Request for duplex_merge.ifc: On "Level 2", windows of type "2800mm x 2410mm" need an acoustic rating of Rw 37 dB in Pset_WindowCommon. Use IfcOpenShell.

First a look at what the model holds.

```python
import ifcopenshell
import ifcopenshell.util.element

model = ifcopenshell.open("duplex_merge.ifc")
print(model.schema)
storey = next(s for s in model.by_type("IfcBuildingStorey") if s.Name == "Level 2")
windows = [e for e in ifcopenshell.util.element.get_decomposition(storey) if e.is_a("IfcWindow")]
seen = {}
for e in windows:
    element_type = ifcopenshell.util.element.get_type(e)
    key = (element_type.Name if element_type != e and element_type else None, ifcopenshell.util.element.get_pset(e, "Pset_WindowCommon", "AcousticRating"))
    seen[key] = seen.get(key, 0) + 1
for (name, value), count in sorted(seen.items(), key=str):
    print(count, "x", name, "|", value)
```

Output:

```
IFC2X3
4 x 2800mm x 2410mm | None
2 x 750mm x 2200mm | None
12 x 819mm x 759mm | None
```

```python
import ifcopenshell
import ifcopenshell.api.pset
import ifcopenshell.util.element

model = ifcopenshell.open("duplex_merge.ifc")

storey = next(s for s in model.by_type("IfcBuildingStorey") if s.Name == "Level 2")
windows = [e for e in ifcopenshell.util.element.get_decomposition(storey) if e.is_a("IfcWindow")]

count = 0
for e in windows:
    element_type = ifcopenshell.util.element.get_type(e)
    if element_type in (None, e) or element_type.Name != "2800mm x 2410mm":
        continue
    # add_pset returns the element's existing set when there is one.
    pset = ifcopenshell.api.pset.add_pset(model, product=e, name="Pset_WindowCommon")
    ifcopenshell.api.pset.edit_pset(model, pset=pset, properties={"AcousticRating": "Rw 37 dB"})
    count += 1

print(count, "windows updated")

model.write("duplex_merge_v2.ifc")
```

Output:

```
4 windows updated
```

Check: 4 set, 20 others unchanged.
